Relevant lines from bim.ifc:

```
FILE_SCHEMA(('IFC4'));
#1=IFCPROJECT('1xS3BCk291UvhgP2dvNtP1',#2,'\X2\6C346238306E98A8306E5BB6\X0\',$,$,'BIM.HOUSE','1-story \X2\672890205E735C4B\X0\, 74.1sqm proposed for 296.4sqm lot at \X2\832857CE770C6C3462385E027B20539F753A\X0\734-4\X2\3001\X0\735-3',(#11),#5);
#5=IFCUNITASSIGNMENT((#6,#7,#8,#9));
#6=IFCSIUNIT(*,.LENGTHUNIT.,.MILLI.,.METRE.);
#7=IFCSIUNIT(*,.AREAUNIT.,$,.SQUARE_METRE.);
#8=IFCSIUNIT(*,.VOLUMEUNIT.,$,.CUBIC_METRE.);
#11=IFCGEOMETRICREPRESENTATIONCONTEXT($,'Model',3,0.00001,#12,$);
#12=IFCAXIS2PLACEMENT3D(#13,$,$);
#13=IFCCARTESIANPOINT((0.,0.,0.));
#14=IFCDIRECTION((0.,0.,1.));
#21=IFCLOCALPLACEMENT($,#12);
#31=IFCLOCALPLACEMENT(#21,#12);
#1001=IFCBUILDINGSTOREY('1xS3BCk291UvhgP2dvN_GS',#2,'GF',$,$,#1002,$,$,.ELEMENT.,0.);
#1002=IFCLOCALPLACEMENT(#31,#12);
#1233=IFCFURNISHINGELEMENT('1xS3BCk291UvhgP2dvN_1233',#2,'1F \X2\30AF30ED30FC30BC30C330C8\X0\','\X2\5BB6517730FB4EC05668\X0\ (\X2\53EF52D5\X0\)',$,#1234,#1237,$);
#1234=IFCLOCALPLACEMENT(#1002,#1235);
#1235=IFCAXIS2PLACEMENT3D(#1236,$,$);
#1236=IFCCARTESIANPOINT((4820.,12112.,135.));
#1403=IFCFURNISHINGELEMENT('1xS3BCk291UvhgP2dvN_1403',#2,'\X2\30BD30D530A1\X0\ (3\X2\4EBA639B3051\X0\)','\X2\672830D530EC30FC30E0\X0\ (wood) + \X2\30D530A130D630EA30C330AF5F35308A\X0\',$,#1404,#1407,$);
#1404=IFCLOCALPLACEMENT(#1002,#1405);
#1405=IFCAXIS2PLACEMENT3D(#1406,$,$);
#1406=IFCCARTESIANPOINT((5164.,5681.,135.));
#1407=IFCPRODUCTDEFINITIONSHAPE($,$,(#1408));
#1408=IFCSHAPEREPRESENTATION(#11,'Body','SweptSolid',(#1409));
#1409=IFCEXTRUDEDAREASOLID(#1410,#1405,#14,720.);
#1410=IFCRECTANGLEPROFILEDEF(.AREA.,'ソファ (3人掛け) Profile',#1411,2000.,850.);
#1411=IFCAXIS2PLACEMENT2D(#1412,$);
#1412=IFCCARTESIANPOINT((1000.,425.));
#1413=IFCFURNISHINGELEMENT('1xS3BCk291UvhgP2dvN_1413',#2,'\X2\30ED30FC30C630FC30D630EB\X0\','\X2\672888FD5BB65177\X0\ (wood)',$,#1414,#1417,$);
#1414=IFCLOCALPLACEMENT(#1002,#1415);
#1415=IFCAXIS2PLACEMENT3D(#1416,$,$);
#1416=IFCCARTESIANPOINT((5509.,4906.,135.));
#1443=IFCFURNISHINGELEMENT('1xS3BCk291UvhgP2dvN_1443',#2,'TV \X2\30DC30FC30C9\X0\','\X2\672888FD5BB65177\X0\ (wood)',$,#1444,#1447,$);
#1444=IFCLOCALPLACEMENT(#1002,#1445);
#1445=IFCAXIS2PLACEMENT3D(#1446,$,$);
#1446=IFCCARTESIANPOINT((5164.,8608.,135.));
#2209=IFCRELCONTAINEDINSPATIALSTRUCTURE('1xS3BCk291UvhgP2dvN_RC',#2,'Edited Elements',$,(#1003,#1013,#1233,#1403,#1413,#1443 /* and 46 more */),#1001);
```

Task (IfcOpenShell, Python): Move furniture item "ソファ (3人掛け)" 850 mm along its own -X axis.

```python
import ifcopenshell
import ifcopenshell.api.geometry
import ifcopenshell.util.placement
import ifcopenshell.util.unit

model = ifcopenshell.open("bim.ifc")
unit_scale = ifcopenshell.util.unit.calculate_unit_scale(model)

item = model.by_id(1403)
matrix = ifcopenshell.util.placement.get_local_placement(item.ObjectPlacement)
matrix[:3, 3] -= matrix[:3, 0] * 0.85 / unit_scale
ifcopenshell.api.geometry.edit_object_placement(model, product=item, matrix=matrix, is_si=False)

print(ifcopenshell.util.placement.get_local_placement(item.ObjectPlacement).round(3) + 0.0)

model.write("bim_v2.ifc")
```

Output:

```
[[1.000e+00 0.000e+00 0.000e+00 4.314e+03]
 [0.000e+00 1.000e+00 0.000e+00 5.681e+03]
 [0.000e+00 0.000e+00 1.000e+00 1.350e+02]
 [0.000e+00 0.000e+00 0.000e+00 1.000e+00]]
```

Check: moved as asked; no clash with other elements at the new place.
